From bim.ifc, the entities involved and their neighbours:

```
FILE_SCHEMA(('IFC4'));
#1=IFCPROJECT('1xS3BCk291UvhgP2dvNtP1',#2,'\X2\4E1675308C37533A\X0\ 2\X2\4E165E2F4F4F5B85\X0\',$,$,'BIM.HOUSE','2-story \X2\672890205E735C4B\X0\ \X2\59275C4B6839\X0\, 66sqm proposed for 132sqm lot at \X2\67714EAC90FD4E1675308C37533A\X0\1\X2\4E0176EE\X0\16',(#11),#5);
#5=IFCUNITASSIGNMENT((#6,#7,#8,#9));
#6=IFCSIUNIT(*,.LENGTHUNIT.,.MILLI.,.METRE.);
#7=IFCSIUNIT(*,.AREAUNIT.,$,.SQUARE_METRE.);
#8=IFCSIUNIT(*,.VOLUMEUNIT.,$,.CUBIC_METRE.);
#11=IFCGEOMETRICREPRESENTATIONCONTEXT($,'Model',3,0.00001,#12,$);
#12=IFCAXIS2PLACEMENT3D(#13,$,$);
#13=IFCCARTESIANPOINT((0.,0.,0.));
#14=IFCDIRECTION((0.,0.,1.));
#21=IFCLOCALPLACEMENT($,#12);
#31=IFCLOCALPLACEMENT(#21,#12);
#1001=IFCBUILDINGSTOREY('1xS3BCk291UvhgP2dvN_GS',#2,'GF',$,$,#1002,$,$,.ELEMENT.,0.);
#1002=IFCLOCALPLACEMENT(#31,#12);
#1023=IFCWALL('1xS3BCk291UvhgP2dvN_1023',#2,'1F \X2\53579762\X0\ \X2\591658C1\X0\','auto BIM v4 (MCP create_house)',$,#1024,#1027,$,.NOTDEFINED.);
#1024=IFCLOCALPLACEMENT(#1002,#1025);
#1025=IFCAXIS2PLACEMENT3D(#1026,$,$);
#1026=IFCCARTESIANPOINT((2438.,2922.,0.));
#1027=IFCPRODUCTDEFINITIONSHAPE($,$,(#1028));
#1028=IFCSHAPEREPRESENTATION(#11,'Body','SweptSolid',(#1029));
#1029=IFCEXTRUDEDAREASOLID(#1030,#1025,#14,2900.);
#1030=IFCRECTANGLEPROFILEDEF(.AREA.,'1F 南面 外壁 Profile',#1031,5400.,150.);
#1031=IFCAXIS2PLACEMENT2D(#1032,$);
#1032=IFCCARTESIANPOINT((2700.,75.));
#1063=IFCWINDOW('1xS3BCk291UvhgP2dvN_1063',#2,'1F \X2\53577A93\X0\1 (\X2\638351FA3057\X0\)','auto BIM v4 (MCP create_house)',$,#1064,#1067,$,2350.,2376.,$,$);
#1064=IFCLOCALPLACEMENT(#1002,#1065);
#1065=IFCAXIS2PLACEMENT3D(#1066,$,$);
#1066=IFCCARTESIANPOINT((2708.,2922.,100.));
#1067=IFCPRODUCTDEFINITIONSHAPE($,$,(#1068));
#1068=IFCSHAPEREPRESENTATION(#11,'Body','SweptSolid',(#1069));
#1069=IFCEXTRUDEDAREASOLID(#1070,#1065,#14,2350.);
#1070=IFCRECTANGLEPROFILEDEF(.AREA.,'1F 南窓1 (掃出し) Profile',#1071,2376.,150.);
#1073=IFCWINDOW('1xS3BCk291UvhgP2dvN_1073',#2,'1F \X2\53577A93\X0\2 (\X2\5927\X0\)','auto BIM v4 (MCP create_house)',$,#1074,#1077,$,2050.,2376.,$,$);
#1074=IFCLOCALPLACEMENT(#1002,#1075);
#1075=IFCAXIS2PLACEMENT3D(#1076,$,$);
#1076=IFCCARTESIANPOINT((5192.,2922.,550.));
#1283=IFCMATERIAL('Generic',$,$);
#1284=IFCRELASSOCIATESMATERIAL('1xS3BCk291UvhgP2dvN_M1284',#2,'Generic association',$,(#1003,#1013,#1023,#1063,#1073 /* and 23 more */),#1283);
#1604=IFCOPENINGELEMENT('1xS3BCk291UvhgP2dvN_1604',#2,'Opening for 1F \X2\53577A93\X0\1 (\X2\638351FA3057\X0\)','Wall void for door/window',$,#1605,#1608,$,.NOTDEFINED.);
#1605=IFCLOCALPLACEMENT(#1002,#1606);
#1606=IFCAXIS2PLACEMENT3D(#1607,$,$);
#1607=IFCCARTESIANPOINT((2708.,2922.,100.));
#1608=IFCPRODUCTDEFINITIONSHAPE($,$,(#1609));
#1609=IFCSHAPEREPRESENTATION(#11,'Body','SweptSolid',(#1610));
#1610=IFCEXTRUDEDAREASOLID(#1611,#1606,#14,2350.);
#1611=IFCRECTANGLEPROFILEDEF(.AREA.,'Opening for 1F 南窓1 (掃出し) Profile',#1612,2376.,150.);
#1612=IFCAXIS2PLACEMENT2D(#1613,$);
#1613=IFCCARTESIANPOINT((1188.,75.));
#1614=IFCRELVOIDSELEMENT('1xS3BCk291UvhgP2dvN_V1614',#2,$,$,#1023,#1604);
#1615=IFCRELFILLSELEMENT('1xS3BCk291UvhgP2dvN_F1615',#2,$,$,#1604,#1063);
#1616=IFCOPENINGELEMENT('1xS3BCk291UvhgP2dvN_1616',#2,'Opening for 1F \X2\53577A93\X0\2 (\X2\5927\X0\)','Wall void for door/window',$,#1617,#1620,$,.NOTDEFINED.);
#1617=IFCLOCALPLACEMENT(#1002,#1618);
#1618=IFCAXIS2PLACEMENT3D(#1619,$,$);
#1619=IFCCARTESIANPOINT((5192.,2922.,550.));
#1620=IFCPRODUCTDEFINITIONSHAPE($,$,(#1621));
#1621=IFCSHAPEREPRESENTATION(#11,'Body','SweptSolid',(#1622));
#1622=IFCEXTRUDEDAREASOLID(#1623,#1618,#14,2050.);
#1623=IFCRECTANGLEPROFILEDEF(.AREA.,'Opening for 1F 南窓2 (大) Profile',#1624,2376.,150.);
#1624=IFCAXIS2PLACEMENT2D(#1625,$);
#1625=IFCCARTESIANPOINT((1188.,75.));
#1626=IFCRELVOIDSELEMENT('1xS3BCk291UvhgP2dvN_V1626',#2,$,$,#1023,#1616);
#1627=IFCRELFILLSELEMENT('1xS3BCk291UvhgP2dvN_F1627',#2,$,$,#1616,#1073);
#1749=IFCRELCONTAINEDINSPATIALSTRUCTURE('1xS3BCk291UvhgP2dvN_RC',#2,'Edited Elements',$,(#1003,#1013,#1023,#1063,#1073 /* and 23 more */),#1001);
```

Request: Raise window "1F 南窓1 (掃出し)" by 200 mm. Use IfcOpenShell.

```python
import numpy as np
import ifcopenshell
import ifcopenshell.api.geometry
import ifcopenshell.util.placement
import ifcopenshell.util.unit

model = ifcopenshell.open("bim.ifc")
unit_scale = ifcopenshell.util.unit.calculate_unit_scale(model)

window = model.by_guid("1xS3BCk291UvhgP2dvN_1063")
opening = window.FillsVoids[0].RelatingOpeningElement
dz = 0.2 / unit_scale

shift = np.array([0.0, 0.0, dz])
# The window is not placed relative to its opening, so move both.
for product in (opening, window):
    matrix = ifcopenshell.util.placement.get_local_placement(product.ObjectPlacement)
    matrix[:3, 3] += shift
    ifcopenshell.api.geometry.edit_object_placement(model, product=product, matrix=matrix, is_si=False)

print(f"moved by {dz * unit_scale:+.3f} m")

model.write("bim-out.ifc")
```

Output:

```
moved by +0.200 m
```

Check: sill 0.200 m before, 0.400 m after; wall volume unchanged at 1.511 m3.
